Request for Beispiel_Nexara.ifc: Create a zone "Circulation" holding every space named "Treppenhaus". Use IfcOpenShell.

First a look at what the model holds.

```python
import ifcopenshell

model = ifcopenshell.open("Beispiel_Nexara.ifc")
print(model.schema)
seen = {}
for space in model.by_type("IfcSpace"):
    seen[space.LongName] = seen.get(space.LongName, 0) + 1
for name, count in sorted(seen.items(), key=str):
    print(count, "x", name)
print("zones:", [z.Name for z in model.by_type("IfcZone")][:20])
```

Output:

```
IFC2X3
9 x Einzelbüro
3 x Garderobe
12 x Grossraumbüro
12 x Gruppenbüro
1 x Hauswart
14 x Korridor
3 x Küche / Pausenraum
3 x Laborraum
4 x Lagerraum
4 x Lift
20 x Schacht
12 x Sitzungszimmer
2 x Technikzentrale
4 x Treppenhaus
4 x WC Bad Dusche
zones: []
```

```python
import ifcopenshell
import ifcopenshell.api.group
import ifcopenshell.api.root

model = ifcopenshell.open("Beispiel_Nexara.ifc")

names = {"Treppenhaus"}
spaces = [s for s in model.by_type("IfcSpace") if s.LongName in names]

zone = ifcopenshell.api.root.create_entity(model, ifc_class="IfcZone", name="Circulation")
ifcopenshell.api.group.assign_group(model, products=spaces, group=zone)
print(len(spaces), "spaces in", zone.Name)

model.write("Beispiel_Nexara-out.ifc")
```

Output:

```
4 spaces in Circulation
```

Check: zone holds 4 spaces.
